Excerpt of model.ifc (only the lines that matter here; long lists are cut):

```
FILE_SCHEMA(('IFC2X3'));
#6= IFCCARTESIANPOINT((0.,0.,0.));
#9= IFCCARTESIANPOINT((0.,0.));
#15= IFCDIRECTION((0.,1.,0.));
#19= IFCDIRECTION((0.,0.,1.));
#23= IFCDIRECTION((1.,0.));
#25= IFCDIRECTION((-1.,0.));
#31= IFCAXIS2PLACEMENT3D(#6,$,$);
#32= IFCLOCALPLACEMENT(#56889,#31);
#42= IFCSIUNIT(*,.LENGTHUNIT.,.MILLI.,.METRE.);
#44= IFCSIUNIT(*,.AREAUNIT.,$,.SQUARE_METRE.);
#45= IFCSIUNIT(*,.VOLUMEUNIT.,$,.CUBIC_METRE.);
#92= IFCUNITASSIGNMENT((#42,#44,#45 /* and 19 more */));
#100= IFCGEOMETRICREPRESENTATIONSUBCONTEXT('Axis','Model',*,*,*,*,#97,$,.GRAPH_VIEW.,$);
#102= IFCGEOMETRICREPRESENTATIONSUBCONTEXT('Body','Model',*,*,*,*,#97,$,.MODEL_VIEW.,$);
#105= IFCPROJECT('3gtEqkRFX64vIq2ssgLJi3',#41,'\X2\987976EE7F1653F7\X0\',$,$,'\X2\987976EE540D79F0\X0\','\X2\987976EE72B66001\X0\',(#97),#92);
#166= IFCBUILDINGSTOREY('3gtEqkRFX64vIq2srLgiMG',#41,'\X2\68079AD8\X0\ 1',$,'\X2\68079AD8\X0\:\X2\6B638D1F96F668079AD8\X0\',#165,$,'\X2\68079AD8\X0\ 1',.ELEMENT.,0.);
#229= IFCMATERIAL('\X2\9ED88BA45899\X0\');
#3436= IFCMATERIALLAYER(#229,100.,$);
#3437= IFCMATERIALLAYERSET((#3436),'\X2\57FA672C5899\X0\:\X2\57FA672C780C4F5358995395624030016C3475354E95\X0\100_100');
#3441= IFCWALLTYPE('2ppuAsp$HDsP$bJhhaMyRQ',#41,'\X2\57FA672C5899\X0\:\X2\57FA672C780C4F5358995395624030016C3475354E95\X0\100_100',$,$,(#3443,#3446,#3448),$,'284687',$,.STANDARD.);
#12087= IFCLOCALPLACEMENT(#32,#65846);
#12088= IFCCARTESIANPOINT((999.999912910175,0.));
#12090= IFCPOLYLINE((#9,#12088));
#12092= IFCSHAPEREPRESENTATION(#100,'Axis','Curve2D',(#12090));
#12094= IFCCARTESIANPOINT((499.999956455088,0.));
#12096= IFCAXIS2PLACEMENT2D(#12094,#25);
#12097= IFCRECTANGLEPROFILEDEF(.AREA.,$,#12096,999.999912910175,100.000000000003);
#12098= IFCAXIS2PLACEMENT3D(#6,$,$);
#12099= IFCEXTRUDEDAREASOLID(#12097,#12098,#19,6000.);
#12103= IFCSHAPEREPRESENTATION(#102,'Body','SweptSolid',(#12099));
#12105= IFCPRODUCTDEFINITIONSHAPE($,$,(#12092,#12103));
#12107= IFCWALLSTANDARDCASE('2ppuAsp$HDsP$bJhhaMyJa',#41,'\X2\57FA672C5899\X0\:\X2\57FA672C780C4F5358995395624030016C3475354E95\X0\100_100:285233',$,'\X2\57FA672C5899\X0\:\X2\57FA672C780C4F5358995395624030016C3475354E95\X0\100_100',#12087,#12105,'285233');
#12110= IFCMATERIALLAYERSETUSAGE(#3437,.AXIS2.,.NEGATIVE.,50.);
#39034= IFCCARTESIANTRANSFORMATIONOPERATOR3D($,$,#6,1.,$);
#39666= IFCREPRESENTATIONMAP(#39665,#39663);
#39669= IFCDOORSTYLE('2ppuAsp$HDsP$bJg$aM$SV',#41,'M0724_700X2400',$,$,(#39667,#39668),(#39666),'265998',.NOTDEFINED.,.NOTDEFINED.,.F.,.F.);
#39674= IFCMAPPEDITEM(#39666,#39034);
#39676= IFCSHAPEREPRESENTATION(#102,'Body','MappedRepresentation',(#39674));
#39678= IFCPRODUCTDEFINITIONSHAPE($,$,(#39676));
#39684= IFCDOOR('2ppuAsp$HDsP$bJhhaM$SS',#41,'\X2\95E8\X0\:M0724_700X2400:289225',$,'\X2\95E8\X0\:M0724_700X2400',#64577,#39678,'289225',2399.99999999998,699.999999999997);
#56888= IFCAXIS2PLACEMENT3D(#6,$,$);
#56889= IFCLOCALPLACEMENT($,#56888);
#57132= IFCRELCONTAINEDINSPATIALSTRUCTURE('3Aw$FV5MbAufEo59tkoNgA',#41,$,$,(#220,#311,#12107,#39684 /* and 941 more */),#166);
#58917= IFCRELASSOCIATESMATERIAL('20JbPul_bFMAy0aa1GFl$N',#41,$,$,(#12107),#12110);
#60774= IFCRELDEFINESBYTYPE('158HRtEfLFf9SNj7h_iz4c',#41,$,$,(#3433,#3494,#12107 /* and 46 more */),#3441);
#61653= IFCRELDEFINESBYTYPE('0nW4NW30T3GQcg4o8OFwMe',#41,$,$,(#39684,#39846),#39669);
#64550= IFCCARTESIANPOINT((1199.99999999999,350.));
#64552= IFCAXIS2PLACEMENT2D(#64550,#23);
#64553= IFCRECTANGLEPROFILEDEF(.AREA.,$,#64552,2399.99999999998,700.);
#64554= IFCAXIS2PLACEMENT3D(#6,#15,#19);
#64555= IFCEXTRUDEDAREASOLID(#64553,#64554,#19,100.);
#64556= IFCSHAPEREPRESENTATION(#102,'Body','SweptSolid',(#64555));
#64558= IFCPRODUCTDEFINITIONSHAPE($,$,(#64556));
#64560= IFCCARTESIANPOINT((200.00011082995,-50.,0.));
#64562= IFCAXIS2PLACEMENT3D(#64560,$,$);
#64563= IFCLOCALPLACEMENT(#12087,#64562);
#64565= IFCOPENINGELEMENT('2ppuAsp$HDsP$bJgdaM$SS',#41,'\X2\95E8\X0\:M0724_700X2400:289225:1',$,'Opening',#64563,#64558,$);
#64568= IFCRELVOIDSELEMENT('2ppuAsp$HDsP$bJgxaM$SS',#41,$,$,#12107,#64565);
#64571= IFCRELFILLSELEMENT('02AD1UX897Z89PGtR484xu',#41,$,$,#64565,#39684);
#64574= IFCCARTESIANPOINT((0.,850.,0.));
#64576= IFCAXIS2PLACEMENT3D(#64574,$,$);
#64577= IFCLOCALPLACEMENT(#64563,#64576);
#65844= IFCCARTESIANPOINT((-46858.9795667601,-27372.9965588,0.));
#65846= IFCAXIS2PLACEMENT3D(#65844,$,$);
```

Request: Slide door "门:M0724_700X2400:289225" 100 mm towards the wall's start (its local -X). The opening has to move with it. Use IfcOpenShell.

```python
import ifcopenshell
import ifcopenshell.api.geometry
import ifcopenshell.util.placement
import ifcopenshell.util.unit

model = ifcopenshell.open("model.ifc")
unit_scale = ifcopenshell.util.unit.calculate_unit_scale(model)

door = model.by_guid("2ppuAsp$HDsP$bJhhaM$SS")
opening = door.FillsVoids[0].RelatingOpeningElement
wall = opening.VoidsElements[0].RelatingBuildingElement

wall_matrix = ifcopenshell.util.placement.get_local_placement(wall.ObjectPlacement)
shift = wall_matrix[:3, 0] * -0.1 / unit_scale
before = ifcopenshell.util.placement.get_local_placement(door.ObjectPlacement)[:3, 3].copy()

# The door is placed relative to its opening, so it follows when the opening moves.
matrix = ifcopenshell.util.placement.get_local_placement(opening.ObjectPlacement)
matrix[:3, 3] += shift
ifcopenshell.api.geometry.edit_object_placement(
    model, product=opening, matrix=matrix, is_si=False, should_transform_children=True
)

after = ifcopenshell.util.placement.get_local_placement(door.ObjectPlacement)[:3, 3]
print("door moved by", (after - before).round(3) + 0.0)

model.write("model_edited.ifc")
```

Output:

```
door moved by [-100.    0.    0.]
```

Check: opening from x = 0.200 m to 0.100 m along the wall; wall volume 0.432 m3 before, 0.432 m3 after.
